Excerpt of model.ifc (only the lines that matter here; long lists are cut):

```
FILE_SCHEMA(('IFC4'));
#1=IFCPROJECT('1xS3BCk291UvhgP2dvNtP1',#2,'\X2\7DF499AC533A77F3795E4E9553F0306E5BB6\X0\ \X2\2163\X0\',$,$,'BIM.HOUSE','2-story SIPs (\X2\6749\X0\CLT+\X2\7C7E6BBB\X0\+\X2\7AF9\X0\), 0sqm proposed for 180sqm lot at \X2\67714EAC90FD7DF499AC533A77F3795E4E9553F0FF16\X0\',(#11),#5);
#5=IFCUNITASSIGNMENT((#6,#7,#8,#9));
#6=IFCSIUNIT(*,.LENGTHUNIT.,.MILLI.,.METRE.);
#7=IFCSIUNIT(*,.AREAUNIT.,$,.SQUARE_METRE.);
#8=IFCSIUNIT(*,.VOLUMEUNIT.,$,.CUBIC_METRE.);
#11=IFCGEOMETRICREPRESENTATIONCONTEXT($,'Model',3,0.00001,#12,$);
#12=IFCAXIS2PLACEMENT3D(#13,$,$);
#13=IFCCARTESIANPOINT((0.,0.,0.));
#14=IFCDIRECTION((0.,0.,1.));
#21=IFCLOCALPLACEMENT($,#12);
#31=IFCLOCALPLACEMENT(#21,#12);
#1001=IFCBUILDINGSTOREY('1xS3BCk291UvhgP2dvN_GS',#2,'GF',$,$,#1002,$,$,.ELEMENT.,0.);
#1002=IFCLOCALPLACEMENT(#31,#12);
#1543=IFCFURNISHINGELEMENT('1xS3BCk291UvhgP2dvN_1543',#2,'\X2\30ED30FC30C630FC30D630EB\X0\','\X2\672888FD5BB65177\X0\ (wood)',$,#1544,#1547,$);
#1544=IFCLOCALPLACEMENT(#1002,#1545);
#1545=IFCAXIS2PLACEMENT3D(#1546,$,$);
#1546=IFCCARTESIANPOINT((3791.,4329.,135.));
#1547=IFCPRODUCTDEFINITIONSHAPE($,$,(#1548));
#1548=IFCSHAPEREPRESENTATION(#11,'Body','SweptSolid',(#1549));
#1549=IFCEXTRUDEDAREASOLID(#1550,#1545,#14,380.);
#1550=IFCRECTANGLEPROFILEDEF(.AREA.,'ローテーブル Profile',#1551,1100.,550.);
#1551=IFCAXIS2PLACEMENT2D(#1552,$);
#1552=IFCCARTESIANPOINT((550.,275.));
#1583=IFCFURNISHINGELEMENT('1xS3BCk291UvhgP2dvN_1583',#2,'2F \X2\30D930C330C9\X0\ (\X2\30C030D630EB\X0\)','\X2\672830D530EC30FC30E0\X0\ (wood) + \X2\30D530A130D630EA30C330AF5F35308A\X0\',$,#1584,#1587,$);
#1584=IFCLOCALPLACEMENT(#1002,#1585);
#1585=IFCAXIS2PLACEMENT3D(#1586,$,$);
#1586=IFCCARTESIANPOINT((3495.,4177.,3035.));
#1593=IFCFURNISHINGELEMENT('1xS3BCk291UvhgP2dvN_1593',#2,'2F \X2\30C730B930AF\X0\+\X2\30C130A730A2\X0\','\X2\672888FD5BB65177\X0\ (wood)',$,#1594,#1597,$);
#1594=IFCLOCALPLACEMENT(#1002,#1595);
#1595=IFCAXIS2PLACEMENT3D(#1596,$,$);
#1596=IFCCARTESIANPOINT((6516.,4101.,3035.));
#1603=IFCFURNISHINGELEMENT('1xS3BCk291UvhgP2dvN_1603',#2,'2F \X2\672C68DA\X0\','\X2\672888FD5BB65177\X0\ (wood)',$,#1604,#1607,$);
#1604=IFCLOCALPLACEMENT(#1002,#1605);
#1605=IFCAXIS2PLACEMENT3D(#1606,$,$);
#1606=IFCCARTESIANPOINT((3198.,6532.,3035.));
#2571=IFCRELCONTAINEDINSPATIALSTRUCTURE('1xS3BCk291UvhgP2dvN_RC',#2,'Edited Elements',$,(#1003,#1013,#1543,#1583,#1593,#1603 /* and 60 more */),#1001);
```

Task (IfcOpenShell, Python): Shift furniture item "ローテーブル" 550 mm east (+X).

```python
import ifcopenshell
import ifcopenshell.api.geometry
import ifcopenshell.util.placement
import ifcopenshell.util.unit

model = ifcopenshell.open("model.ifc")
unit_scale = ifcopenshell.util.unit.calculate_unit_scale(model)

item = model.by_id(1543)
matrix = ifcopenshell.util.placement.get_local_placement(item.ObjectPlacement)
matrix[0, 3] += 0.55 / unit_scale
ifcopenshell.api.geometry.edit_object_placement(model, product=item, matrix=matrix, is_si=False)

print(ifcopenshell.util.placement.get_local_placement(item.ObjectPlacement).round(3) + 0.0)

model.write("model_v2.ifc")
```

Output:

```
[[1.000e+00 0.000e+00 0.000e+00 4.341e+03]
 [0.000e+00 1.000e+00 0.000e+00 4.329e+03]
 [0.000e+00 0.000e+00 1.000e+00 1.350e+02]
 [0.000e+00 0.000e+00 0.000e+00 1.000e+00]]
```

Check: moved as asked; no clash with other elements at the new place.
